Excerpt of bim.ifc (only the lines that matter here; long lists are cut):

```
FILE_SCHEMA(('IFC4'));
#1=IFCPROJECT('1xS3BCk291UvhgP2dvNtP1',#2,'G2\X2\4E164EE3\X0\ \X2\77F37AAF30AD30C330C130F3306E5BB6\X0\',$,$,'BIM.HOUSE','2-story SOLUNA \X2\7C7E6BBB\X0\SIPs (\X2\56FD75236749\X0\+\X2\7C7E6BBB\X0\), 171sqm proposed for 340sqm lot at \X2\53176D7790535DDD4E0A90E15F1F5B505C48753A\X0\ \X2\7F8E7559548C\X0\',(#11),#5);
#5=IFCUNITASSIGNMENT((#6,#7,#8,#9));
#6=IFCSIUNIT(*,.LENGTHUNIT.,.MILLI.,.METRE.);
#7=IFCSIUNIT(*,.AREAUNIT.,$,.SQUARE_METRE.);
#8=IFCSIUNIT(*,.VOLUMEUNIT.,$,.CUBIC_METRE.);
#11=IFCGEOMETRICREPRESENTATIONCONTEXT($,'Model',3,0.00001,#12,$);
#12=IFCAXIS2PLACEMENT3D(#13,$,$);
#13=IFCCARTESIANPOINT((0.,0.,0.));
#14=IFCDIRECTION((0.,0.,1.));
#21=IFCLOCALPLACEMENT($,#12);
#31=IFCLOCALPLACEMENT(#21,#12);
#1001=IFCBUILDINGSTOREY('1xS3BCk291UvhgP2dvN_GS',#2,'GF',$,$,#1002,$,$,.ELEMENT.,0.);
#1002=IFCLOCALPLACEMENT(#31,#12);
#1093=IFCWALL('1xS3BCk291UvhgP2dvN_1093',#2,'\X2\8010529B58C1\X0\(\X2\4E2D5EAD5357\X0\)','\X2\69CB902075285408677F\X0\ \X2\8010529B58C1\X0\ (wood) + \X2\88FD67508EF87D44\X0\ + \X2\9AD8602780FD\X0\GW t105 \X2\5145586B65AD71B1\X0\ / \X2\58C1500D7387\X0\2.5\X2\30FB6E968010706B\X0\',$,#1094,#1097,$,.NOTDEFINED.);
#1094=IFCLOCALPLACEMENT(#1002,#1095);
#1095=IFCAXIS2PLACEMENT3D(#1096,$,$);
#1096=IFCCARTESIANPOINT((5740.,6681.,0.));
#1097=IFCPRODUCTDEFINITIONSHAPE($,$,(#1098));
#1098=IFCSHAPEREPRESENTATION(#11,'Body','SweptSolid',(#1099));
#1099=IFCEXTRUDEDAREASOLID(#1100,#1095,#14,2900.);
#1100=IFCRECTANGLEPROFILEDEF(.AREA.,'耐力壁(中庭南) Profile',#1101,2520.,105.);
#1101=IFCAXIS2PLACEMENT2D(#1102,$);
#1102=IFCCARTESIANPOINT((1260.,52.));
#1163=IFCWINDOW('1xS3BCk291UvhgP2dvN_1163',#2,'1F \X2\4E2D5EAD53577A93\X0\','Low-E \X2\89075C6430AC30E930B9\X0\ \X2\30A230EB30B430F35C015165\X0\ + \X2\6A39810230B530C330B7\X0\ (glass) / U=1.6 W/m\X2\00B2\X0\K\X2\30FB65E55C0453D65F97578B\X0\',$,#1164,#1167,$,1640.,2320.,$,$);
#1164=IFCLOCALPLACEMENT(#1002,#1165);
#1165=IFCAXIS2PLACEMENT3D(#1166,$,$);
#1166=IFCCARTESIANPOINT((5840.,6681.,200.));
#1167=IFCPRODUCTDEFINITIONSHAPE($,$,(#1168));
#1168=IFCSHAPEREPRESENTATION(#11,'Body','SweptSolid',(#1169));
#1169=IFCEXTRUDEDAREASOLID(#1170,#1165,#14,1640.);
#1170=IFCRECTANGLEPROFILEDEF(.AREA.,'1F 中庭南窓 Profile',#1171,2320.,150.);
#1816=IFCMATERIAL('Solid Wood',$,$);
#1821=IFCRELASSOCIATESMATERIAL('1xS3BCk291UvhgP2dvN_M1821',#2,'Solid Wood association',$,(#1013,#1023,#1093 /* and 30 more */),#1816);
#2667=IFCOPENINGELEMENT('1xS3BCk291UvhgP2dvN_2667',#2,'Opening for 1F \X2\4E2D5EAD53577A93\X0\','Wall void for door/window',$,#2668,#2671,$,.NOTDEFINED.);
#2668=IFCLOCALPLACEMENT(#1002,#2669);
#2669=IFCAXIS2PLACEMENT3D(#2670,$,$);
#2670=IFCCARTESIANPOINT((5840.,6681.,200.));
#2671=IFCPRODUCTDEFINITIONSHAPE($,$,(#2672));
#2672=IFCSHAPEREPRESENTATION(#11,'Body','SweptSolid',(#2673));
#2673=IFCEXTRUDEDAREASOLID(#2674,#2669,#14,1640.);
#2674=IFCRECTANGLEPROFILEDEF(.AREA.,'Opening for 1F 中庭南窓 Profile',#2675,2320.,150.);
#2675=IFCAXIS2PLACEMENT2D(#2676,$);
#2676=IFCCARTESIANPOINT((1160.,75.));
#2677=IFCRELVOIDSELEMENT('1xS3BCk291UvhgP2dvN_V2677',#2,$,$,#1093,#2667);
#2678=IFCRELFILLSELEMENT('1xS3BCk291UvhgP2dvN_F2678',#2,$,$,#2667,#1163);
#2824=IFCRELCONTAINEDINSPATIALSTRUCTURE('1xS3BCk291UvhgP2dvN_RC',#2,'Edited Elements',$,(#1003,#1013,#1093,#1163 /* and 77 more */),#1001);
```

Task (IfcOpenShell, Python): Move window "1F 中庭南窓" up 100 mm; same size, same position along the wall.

```python
import numpy as np
import ifcopenshell
import ifcopenshell.api.geometry
import ifcopenshell.util.placement
import ifcopenshell.util.unit

model = ifcopenshell.open("bim.ifc")
unit_scale = ifcopenshell.util.unit.calculate_unit_scale(model)

window = model.by_guid("1xS3BCk291UvhgP2dvN_1163")
opening = window.FillsVoids[0].RelatingOpeningElement
dz = 100.0

shift = np.array([0.0, 0.0, dz])
# The window is not placed relative to its opening, so move both.
for product in (opening, window):
    matrix = ifcopenshell.util.placement.get_local_placement(product.ObjectPlacement)
    matrix[:3, 3] += shift
    ifcopenshell.api.geometry.edit_object_placement(model, product=product, matrix=matrix, is_si=False)

print(f"moved by {dz * unit_scale:+.3f} m")

model.write("bim_edited.ifc")
```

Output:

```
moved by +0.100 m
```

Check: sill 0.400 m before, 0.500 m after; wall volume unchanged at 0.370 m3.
